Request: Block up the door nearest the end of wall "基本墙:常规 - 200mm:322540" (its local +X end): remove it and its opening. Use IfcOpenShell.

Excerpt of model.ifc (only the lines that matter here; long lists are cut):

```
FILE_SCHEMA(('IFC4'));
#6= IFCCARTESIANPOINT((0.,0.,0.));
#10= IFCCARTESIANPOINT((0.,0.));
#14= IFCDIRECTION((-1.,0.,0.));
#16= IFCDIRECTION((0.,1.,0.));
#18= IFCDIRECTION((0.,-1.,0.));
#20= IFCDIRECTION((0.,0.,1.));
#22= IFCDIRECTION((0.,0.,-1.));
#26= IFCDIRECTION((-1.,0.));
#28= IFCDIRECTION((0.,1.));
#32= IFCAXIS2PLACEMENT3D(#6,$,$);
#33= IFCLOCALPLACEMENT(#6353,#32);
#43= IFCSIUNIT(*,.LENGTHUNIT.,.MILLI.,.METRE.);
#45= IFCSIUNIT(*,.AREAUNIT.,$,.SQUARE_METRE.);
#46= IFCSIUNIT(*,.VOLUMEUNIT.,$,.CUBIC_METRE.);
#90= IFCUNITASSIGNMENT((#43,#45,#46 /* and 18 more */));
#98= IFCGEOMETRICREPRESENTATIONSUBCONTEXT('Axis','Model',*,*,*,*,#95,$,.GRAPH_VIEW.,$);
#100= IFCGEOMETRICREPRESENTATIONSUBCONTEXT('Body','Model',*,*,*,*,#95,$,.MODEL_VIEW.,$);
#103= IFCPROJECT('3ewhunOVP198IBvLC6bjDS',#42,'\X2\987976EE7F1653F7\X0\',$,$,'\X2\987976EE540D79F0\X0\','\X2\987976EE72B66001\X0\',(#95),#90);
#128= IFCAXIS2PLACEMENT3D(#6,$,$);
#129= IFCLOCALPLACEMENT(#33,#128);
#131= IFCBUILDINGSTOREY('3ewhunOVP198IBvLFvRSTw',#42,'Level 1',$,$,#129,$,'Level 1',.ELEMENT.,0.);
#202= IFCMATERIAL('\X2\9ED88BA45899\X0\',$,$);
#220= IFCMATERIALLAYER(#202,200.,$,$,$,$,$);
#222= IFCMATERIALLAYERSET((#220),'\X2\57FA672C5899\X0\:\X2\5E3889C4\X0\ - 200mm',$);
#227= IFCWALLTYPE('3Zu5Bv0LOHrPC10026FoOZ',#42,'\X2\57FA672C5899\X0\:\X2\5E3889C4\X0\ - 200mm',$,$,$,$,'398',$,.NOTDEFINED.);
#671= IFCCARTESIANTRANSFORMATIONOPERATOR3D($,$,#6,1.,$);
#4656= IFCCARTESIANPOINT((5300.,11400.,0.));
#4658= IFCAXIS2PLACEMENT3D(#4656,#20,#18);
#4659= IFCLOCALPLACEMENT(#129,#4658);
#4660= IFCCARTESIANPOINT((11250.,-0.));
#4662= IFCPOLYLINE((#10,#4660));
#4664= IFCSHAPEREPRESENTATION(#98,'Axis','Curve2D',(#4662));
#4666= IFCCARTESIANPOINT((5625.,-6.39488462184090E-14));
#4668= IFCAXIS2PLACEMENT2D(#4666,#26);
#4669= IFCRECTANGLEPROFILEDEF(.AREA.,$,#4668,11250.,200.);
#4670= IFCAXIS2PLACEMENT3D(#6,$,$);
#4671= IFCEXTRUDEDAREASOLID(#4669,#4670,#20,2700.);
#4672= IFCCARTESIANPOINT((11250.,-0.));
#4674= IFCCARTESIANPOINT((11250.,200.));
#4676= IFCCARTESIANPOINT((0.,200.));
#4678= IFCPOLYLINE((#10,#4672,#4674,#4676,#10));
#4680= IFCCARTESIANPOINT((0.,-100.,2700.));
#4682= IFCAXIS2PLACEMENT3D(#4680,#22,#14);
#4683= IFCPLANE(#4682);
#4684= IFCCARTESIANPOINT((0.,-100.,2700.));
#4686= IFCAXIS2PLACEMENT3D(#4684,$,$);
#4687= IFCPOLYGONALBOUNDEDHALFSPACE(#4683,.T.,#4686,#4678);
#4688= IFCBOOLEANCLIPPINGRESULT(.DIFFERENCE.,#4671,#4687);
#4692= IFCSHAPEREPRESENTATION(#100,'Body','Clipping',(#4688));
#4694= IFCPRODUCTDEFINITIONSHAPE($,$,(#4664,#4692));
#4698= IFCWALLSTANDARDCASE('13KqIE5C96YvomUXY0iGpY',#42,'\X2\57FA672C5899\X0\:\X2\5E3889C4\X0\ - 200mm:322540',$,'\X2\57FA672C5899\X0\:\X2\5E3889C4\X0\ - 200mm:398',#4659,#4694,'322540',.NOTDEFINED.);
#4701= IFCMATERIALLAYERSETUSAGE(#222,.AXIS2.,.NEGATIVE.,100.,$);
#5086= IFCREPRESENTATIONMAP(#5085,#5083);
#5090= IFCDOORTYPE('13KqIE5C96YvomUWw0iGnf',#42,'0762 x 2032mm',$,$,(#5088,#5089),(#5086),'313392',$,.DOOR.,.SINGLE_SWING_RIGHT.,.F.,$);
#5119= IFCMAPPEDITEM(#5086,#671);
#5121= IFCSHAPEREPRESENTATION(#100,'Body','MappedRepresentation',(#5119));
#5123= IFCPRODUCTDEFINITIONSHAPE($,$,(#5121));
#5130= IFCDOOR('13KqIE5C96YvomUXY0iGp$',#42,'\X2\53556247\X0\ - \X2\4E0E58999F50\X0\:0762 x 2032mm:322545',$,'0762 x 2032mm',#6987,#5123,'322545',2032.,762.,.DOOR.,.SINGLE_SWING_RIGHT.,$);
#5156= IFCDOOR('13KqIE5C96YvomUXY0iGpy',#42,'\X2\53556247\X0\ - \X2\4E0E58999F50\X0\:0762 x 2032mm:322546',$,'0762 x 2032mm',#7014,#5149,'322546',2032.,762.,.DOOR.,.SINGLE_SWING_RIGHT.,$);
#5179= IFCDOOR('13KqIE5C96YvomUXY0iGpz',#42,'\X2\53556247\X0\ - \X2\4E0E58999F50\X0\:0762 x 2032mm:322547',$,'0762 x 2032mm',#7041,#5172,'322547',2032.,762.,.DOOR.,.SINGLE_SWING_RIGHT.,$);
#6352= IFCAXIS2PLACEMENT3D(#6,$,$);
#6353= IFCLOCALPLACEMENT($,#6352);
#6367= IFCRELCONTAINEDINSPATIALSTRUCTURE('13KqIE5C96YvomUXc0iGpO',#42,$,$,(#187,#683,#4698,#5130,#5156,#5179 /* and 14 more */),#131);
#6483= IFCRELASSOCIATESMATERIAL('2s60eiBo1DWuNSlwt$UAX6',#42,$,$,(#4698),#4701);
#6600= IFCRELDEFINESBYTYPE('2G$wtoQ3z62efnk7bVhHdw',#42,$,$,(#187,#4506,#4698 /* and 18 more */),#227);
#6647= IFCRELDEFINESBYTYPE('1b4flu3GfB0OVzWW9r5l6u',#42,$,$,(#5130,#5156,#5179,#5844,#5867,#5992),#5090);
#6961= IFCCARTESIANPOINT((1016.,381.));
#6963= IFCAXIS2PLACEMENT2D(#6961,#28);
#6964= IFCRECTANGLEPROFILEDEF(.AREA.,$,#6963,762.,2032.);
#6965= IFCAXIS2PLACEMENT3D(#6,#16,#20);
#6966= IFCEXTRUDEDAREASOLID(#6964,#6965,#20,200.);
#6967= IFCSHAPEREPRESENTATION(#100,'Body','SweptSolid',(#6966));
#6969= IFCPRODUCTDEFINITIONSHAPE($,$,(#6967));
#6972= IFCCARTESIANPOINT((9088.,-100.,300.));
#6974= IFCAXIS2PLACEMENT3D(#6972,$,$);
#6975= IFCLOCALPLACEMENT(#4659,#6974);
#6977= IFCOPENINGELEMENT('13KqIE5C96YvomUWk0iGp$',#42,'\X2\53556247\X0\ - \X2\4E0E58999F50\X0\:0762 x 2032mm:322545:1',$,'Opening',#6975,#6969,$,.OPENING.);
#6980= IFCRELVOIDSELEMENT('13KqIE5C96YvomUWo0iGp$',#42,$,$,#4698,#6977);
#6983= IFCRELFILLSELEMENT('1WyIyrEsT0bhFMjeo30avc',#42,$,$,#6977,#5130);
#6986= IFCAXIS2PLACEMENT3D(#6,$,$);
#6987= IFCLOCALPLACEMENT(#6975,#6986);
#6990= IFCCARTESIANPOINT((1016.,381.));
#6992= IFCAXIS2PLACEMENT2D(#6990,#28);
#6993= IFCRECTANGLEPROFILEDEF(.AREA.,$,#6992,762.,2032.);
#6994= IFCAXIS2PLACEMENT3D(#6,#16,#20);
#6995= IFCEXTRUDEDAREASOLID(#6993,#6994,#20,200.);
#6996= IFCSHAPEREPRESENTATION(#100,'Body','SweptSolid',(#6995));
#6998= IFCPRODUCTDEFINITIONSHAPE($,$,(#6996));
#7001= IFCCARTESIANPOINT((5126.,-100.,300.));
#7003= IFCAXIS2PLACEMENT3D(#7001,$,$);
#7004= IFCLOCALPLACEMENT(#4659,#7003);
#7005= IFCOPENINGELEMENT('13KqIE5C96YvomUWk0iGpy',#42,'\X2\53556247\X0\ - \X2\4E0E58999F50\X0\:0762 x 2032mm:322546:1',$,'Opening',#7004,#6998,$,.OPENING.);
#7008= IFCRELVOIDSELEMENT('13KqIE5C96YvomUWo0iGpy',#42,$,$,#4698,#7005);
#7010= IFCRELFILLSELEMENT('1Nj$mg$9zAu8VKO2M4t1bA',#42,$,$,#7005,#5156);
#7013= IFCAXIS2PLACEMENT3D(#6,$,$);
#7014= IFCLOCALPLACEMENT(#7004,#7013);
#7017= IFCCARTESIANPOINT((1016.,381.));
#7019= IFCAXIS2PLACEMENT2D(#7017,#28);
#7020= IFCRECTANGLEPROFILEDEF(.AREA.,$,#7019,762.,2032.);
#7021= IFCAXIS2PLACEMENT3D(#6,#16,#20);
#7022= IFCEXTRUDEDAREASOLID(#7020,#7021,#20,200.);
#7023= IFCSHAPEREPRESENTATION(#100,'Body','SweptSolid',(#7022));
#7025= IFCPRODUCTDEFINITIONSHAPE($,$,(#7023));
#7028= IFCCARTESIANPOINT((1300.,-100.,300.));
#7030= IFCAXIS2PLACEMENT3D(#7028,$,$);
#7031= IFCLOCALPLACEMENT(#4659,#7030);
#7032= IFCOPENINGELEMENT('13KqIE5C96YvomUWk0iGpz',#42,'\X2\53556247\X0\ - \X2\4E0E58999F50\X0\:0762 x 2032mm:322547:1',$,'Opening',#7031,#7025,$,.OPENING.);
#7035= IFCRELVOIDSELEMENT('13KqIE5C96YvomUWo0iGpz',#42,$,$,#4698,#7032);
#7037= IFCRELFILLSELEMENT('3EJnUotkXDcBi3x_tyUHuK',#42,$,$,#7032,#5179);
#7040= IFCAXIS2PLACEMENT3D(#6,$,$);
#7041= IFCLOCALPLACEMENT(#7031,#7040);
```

```python
import ifcopenshell
import ifcopenshell.api.feature
import ifcopenshell.api.root
import ifcopenshell.geom
import ifcopenshell.util.shape

model = ifcopenshell.open("model.ifc")
settings = ifcopenshell.geom.settings()


def volume(element):
    """Net volume in cubic metres, openings subtracted."""
    shape = ifcopenshell.geom.create_shape(settings, element)
    return ifcopenshell.util.shape.get_volume(shape.geometry)


door = model.by_guid("13KqIE5C96YvomUXY0iGp$")
opening = door.FillsVoids[0].RelatingOpeningElement
wall = opening.VoidsElements[0].RelatingBuildingElement
before = volume(wall)

ifcopenshell.api.root.remove_product(model, product=door)
ifcopenshell.api.feature.remove_feature(model, feature=opening)

after = volume(wall)

print(f"wall volume {before:.3f} -> {after:.3f} m3")

model.write("model_edited.ifc")
```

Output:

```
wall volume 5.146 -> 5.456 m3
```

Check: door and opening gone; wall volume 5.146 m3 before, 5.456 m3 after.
